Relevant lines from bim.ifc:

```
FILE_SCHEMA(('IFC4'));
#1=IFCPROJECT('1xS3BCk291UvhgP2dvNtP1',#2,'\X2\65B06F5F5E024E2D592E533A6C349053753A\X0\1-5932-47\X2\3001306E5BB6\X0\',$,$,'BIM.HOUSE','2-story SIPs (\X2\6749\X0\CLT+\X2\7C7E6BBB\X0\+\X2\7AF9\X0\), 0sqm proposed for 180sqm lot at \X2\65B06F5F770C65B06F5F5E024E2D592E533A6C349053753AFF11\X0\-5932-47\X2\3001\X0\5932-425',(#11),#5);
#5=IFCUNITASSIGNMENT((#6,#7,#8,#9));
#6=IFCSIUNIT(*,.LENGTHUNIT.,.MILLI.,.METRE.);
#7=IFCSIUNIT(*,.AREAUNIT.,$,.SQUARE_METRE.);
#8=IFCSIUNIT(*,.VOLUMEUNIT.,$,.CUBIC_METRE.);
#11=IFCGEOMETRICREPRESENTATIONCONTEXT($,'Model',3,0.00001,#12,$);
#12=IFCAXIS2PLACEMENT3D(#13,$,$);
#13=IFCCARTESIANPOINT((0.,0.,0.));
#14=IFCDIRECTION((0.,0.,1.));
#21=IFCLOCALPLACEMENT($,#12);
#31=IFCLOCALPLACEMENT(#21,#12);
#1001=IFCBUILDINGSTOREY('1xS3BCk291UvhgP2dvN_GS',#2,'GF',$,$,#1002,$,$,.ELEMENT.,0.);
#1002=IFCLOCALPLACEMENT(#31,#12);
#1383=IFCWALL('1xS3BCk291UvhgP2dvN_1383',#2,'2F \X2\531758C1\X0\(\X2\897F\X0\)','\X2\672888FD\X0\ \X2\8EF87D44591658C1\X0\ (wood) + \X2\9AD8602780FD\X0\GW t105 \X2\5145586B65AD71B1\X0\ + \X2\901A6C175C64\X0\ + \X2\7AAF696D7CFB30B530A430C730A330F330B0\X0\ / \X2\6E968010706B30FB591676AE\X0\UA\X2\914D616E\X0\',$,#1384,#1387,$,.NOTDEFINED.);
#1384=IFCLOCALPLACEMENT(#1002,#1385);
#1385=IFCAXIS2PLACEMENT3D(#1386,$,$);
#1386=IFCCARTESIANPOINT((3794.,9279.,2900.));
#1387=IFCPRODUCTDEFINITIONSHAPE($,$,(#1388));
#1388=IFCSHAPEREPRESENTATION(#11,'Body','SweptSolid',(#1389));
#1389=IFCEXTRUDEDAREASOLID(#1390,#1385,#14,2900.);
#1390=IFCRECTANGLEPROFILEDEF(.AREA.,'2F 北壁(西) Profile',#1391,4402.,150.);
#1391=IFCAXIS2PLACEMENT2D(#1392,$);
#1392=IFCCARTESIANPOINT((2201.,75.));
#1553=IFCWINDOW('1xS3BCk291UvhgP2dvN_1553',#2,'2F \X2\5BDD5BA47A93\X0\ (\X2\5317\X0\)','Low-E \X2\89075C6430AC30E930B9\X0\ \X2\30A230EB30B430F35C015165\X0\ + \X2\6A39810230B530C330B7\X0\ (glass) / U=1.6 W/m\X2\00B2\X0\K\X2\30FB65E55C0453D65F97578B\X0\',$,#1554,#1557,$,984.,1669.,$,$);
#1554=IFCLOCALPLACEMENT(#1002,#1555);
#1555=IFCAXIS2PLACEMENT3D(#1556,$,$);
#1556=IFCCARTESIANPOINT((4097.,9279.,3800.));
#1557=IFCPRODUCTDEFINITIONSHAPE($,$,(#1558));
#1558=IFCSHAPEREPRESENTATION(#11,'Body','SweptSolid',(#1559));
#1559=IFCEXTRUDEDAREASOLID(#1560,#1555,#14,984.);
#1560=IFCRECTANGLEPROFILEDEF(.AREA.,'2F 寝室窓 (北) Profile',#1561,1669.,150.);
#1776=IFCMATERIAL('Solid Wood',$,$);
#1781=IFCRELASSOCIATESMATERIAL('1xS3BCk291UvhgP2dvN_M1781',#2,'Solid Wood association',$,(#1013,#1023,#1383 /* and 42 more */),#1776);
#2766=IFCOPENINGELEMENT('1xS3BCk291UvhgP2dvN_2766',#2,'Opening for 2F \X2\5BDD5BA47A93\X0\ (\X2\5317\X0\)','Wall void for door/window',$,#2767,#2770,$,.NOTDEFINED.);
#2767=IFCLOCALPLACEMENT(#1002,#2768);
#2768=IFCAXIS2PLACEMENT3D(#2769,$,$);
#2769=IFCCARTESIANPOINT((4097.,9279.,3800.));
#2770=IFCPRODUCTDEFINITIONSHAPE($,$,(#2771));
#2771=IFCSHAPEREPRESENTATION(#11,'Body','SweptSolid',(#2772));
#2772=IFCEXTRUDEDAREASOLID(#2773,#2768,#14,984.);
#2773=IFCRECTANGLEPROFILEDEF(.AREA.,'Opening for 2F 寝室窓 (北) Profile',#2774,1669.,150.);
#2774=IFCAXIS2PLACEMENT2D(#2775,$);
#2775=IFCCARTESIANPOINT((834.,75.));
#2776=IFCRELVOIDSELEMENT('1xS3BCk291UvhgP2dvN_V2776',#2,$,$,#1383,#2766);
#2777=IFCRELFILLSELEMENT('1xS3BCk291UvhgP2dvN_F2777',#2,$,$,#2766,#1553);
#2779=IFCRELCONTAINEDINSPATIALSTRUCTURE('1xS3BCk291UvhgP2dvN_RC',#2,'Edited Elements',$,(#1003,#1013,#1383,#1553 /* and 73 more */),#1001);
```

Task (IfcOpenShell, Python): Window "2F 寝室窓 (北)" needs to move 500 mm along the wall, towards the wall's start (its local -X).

```python
import ifcopenshell
import ifcopenshell.api.geometry
import ifcopenshell.util.placement
import ifcopenshell.util.unit

model = ifcopenshell.open("bim.ifc")
unit_scale = ifcopenshell.util.unit.calculate_unit_scale(model)

window = model.by_id(1553)
opening = window.FillsVoids[0].RelatingOpeningElement
wall = opening.VoidsElements[0].RelatingBuildingElement

wall_matrix = ifcopenshell.util.placement.get_local_placement(wall.ObjectPlacement)
shift = wall_matrix[:3, 0] * -0.5 / unit_scale
before = ifcopenshell.util.placement.get_local_placement(window.ObjectPlacement)[:3, 3].copy()

# The window is not placed relative to its opening, so move both.
for product in (opening, window):
    matrix = ifcopenshell.util.placement.get_local_placement(product.ObjectPlacement)
    matrix[:3, 3] += shift
    ifcopenshell.api.geometry.edit_object_placement(model, product=product, matrix=matrix, is_si=False)

after = ifcopenshell.util.placement.get_local_placement(window.ObjectPlacement)[:3, 3]
print("window moved by", (after - before).round(3) + 0.0)

model.write("bim_rev.ifc")
```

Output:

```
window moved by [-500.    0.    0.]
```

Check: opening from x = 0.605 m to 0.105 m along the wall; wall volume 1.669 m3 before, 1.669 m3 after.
